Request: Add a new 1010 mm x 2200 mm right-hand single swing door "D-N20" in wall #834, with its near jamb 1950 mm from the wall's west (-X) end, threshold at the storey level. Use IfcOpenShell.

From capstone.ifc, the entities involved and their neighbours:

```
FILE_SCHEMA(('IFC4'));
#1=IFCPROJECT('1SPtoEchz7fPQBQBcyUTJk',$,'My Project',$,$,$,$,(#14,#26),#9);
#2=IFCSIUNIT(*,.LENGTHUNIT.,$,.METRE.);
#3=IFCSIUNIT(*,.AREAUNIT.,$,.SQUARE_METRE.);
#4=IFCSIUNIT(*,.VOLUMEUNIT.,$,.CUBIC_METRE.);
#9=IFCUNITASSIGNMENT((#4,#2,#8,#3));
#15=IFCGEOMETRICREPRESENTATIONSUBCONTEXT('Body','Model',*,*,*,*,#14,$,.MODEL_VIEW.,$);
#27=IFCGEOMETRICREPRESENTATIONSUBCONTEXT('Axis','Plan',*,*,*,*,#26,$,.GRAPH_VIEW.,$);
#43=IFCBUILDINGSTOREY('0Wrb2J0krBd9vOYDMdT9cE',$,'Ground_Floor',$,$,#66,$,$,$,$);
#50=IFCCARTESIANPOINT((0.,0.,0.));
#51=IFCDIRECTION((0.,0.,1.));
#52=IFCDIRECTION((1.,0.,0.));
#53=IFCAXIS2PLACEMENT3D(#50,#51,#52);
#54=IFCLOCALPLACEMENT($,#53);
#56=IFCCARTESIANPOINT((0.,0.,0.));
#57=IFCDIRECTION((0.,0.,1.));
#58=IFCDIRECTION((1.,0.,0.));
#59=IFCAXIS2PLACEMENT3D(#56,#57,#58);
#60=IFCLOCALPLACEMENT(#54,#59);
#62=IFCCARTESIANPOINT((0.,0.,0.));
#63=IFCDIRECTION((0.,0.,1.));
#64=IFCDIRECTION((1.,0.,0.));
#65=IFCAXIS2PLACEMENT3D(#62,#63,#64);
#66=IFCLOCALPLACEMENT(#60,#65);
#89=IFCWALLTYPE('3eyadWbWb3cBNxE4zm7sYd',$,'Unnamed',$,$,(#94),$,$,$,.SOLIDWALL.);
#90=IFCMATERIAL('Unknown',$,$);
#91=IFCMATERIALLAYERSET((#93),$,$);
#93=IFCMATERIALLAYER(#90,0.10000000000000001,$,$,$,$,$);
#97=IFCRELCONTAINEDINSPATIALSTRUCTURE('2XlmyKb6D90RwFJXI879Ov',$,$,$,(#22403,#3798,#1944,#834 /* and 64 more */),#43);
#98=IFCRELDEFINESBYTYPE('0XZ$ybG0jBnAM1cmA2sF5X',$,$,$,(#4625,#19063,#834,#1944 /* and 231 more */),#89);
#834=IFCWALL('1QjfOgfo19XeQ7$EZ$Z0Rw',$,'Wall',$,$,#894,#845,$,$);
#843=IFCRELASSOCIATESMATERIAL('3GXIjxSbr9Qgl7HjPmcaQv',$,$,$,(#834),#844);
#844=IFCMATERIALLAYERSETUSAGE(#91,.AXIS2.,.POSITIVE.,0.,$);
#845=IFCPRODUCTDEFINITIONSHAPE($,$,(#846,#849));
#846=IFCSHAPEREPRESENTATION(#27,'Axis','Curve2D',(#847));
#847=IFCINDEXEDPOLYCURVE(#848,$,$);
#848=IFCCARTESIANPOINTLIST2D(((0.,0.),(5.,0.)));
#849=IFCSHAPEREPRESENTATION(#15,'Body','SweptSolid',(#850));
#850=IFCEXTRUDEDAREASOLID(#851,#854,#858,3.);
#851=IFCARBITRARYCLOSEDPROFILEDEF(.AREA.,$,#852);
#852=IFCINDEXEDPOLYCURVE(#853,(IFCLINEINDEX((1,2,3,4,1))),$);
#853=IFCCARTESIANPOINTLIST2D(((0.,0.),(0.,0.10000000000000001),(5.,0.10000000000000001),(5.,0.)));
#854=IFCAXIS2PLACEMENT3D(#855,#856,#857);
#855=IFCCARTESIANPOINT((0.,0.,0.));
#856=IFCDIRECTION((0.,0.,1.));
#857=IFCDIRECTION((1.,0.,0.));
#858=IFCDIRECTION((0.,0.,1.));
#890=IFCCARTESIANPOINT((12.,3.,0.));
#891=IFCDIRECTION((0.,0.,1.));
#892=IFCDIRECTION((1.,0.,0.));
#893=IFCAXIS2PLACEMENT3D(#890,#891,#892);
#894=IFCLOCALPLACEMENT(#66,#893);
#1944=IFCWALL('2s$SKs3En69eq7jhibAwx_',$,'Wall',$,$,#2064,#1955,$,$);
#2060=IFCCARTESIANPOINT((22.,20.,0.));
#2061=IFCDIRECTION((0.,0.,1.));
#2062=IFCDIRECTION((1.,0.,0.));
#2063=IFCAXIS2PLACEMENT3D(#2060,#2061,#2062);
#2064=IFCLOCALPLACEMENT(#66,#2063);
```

```python
import numpy as np
import ifcopenshell
import ifcopenshell.api.feature
import ifcopenshell.api.geometry
import ifcopenshell.api.root
import ifcopenshell.api.spatial
import ifcopenshell.geom
import ifcopenshell.util.element
import ifcopenshell.util.placement
import ifcopenshell.util.representation
import ifcopenshell.util.shape
import ifcopenshell.util.unit

model = ifcopenshell.open("capstone.ifc")
unit_scale = ifcopenshell.util.unit.calculate_unit_scale(model)
settings = ifcopenshell.geom.settings()


def volume(element):
    """Net volume in cubic metres, openings subtracted."""
    shape = ifcopenshell.geom.create_shape(settings, element)
    return ifcopenshell.util.shape.get_volume(shape.geometry)


wall = model.by_guid("1QjfOgfo19XeQ7$EZ$Z0Rw")
storey = ifcopenshell.util.element.get_container(wall, ifc_class="IfcBuildingStorey")
context = ifcopenshell.util.representation.get_context(model, "Model", "Body", "MODEL_VIEW")
before = volume(wall)

width, height, from_end, sill = 1.01, 2.2, 1.95, 0.0  # metres

# The wall runs along its own X axis, and the end named is its -X end.
wall_shape = ifcopenshell.geom.create_shape(settings, wall)
x, y, z = ifcopenshell.util.shape.get_vertices(wall_shape.geometry).T
start = x.min() + from_end
face, thickness = float(y.min()), float(y.max() - y.min())
wall_matrix = ifcopenshell.util.placement.get_local_placement(wall.ObjectPlacement)
level = ifcopenshell.util.placement.get_local_placement(storey.ObjectPlacement)[2, 3]


def in_wall(x, y):
    """Placement at x, y metres in the wall's axes, at sill height."""
    matrix = wall_matrix.copy()
    matrix[:, 3] = wall_matrix @ np.array([x / unit_scale, y / unit_scale, 0.0, 1.0])
    matrix[2, 3] = level + sill / unit_scale
    return matrix


# Opening: a box that overshoots both wall faces by 50 mm.
opening = ifcopenshell.api.root.create_entity(model, ifc_class="IfcOpeningElement", predefined_type="OPENING")
box = ifcopenshell.api.geometry.add_wall_representation(
    model, context=context, length=width, height=height, thickness=thickness + 0.1
)
ifcopenshell.api.geometry.assign_representation(model, product=opening, representation=box)
ifcopenshell.api.geometry.edit_object_placement(model, product=opening, matrix=in_wall(start, face - 0.05), is_si=False)
ifcopenshell.api.feature.add_feature(model, feature=opening, element=wall)

door = ifcopenshell.api.root.create_entity(model, ifc_class="IfcDoor", name="D-N20", predefined_type="DOOR")
door.OverallWidth, door.OverallHeight = width / unit_scale, height / unit_scale
door.OperationType = "SINGLE_SWING_RIGHT"
body = ifcopenshell.api.geometry.add_door_representation(
    model,
    context=context,
    overall_width=door.OverallWidth,
    overall_height=door.OverallHeight,
    operation_type="SINGLE_SWING_RIGHT",
    lining_properties={"LiningDepth": thickness / unit_scale, "ThresholdDepth": thickness / unit_scale},
)
ifcopenshell.api.geometry.assign_representation(model, product=door, representation=body)
ifcopenshell.api.spatial.assign_container(model, products=[door], relating_structure=storey)
ifcopenshell.api.feature.add_filling(model, opening=opening, element=door)

# The lining spans the wall, so the door starts at the wall face.
ifcopenshell.api.geometry.edit_object_placement(model, product=door, matrix=in_wall(start, face), is_si=False)

after = volume(wall)

print(f"wall volume {before:.3f} -> {after:.3f} m3")

model.write("capstone_v2.ifc")
```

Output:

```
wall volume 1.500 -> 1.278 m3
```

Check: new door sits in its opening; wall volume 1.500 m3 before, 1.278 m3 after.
